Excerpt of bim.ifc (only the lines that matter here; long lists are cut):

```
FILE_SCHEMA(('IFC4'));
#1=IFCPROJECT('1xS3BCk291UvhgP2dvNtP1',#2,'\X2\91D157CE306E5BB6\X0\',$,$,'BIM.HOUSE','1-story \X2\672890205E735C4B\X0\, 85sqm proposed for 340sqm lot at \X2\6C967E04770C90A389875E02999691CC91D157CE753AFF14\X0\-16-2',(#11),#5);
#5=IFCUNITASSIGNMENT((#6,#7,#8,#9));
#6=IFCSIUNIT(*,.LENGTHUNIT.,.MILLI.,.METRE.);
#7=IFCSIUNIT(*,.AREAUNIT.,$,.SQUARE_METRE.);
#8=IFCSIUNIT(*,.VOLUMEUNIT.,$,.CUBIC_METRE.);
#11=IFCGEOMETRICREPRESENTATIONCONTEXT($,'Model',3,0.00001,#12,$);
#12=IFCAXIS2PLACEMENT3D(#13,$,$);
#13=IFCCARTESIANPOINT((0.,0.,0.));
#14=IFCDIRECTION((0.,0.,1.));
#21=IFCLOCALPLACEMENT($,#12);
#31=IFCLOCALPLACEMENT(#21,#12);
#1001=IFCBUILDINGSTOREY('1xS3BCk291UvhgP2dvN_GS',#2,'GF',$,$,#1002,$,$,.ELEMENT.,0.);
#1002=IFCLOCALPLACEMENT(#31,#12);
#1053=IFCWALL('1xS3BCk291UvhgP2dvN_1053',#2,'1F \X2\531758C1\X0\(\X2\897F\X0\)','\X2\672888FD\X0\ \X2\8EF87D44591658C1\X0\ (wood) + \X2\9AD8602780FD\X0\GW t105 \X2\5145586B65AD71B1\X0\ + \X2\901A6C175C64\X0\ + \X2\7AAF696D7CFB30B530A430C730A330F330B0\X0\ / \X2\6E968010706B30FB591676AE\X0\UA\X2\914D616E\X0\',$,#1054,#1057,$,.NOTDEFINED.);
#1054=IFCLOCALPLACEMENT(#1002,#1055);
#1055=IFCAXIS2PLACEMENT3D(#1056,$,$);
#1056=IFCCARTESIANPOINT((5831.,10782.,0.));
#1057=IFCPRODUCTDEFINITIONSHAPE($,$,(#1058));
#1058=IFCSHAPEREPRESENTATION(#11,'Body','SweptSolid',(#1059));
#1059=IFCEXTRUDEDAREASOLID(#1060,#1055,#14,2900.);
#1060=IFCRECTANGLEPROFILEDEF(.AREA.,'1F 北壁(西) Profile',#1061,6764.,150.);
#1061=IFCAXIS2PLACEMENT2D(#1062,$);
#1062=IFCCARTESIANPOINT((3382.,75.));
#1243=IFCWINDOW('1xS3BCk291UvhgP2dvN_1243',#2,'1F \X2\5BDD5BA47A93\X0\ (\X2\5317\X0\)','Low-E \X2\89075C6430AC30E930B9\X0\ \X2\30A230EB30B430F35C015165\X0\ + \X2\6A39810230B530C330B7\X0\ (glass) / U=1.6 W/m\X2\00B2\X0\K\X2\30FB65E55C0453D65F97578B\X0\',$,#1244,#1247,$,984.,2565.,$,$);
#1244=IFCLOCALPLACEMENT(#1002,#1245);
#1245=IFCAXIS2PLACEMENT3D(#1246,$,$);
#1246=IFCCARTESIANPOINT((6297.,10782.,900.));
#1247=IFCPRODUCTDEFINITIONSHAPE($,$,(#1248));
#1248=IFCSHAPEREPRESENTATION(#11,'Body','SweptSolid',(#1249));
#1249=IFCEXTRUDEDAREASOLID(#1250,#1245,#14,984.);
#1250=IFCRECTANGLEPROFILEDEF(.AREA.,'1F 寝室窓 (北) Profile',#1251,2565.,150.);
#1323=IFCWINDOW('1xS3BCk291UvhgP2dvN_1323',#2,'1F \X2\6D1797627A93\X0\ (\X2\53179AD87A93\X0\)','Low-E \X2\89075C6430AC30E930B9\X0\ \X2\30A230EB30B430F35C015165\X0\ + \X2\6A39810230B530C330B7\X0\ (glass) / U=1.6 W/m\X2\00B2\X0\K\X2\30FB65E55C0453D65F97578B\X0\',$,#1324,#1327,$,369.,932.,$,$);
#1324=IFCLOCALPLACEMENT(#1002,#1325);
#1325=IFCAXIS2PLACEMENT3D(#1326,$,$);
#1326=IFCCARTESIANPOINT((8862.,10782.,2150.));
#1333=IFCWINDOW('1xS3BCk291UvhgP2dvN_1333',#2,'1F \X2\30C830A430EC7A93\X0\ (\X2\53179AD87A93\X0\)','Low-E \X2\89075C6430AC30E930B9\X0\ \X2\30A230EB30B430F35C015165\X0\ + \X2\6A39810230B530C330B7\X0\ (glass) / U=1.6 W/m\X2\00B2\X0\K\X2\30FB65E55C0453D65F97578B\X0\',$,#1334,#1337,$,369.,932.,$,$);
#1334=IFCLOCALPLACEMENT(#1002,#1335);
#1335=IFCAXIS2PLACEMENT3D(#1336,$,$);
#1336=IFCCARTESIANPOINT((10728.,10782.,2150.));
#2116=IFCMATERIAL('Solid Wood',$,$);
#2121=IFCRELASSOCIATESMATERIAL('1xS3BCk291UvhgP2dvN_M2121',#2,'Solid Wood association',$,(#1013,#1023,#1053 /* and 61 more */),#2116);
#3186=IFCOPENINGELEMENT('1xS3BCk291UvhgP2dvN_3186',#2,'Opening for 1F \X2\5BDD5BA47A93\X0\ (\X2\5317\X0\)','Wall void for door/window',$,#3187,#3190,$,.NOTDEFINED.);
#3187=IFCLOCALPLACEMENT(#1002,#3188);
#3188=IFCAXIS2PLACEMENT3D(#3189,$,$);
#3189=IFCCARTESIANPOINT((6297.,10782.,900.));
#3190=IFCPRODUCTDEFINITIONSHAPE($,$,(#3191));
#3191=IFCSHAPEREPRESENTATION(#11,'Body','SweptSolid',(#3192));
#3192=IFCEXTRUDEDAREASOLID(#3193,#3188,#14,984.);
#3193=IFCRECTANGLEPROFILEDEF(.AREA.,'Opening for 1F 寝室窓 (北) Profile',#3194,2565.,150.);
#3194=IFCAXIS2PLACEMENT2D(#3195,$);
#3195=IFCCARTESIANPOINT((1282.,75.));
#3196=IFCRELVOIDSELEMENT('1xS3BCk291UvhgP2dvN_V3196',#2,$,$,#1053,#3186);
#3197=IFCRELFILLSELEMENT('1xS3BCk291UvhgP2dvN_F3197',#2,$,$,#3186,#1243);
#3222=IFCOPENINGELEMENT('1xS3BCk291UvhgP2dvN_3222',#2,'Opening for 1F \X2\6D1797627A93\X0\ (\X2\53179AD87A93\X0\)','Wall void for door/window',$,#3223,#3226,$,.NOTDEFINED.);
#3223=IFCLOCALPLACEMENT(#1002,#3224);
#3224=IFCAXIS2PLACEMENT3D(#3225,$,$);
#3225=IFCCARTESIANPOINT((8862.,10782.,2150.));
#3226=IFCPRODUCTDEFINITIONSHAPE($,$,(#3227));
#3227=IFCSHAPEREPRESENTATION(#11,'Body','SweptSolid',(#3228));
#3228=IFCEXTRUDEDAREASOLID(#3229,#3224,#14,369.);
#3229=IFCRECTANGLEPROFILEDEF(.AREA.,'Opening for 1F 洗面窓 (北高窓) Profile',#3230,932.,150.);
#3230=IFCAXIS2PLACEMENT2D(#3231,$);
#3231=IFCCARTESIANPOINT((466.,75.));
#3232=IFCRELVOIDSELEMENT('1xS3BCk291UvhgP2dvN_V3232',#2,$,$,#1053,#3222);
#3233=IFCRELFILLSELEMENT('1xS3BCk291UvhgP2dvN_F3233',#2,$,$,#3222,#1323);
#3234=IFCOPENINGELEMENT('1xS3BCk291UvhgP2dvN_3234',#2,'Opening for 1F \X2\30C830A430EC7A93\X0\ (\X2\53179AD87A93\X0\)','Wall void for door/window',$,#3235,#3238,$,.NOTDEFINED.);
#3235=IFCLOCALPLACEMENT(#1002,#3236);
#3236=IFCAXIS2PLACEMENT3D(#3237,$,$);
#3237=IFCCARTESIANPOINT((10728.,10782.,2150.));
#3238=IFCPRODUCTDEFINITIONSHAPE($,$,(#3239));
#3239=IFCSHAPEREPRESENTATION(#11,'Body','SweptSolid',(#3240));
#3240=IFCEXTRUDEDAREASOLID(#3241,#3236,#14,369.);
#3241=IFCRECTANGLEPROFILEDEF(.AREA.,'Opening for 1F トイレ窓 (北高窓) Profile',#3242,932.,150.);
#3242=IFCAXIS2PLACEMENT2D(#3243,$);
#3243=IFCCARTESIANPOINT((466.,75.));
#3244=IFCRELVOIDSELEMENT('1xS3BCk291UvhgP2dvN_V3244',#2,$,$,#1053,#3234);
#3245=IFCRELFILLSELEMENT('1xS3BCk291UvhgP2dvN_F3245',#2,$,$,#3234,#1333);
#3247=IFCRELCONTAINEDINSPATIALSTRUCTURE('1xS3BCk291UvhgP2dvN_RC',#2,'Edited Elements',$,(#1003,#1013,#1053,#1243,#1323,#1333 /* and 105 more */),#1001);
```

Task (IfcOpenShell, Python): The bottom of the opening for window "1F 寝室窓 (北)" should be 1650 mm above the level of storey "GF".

```python
import numpy as np
import ifcopenshell
import ifcopenshell.api.geometry
import ifcopenshell.geom
import ifcopenshell.util.element
import ifcopenshell.util.placement
import ifcopenshell.util.shape
import ifcopenshell.util.unit

model = ifcopenshell.open("bim.ifc")
unit_scale = ifcopenshell.util.unit.calculate_unit_scale(model)

window = model.by_guid("1xS3BCk291UvhgP2dvN_1243")
opening = window.FillsVoids[0].RelatingOpeningElement
storey = ifcopenshell.util.element.get_container(window, ifc_class="IfcBuildingStorey")
level = ifcopenshell.util.placement.get_local_placement(storey.ObjectPlacement)[2, 3]

# The opening's origin need not be at the sill, so measure its lowest point.
shape = ifcopenshell.geom.create_shape(ifcopenshell.geom.settings(), opening)
bottom = ifcopenshell.util.shape.get_shape_bottom_elevation(shape, shape.geometry) / unit_scale
dz = level + 1.65 / unit_scale - bottom

shift = np.array([0.0, 0.0, dz])
# The window is not placed relative to its opening, so move both.
for product in (opening, window):
    matrix = ifcopenshell.util.placement.get_local_placement(product.ObjectPlacement)
    matrix[:3, 3] += shift
    ifcopenshell.api.geometry.edit_object_placement(model, product=product, matrix=matrix, is_si=False)

print(f"moved by {dz * unit_scale:+.3f} m")

model.write("bim_v2.ifc")
```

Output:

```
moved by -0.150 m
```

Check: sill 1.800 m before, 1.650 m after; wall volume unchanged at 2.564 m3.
